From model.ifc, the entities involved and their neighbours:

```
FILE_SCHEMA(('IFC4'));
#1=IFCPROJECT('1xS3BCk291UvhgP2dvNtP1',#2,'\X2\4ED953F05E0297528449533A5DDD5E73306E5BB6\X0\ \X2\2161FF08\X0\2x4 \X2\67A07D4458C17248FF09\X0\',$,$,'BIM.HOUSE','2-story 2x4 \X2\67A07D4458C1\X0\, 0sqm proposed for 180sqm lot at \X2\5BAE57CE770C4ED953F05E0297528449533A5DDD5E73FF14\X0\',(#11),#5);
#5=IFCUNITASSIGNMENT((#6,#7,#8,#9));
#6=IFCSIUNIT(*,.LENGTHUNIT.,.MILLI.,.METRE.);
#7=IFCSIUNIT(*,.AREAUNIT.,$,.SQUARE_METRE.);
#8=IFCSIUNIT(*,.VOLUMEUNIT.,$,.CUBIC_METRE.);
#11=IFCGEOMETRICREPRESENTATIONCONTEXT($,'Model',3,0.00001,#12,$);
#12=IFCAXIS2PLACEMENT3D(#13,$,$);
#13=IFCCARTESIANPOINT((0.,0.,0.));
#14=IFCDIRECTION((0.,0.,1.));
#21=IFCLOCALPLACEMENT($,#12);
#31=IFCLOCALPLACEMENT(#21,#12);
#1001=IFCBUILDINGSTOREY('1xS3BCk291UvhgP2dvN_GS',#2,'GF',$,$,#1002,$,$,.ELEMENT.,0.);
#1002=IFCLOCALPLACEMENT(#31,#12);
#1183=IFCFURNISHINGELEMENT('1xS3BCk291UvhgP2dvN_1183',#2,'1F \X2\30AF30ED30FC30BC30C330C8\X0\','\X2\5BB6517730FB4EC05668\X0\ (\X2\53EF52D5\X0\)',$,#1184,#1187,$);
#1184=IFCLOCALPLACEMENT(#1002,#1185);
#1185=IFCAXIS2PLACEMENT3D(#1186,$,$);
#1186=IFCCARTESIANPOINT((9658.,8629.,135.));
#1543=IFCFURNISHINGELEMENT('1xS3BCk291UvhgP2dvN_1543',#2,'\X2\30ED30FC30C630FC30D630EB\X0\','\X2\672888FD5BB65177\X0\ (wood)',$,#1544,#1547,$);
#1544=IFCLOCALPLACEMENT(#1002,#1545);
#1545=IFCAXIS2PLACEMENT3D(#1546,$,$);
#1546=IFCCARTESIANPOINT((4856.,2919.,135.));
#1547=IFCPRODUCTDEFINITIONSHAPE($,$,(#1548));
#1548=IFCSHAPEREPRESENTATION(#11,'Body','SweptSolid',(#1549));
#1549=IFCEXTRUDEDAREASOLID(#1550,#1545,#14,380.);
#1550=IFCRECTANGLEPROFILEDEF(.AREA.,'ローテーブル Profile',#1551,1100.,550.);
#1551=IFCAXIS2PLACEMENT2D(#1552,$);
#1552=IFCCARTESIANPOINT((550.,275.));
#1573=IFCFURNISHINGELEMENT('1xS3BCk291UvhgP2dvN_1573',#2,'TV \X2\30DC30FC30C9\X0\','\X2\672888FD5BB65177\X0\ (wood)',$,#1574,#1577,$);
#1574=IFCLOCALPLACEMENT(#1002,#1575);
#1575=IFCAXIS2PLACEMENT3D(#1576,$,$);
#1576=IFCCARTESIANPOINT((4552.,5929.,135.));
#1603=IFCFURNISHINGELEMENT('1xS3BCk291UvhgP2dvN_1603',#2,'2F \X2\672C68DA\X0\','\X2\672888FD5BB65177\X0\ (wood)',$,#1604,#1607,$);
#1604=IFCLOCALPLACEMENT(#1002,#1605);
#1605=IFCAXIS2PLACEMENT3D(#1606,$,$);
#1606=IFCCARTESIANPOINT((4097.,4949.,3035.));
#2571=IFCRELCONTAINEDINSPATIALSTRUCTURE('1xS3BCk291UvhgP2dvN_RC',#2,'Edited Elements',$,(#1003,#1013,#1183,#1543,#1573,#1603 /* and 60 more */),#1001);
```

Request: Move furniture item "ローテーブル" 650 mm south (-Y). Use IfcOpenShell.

```python
import ifcopenshell
import ifcopenshell.api.geometry
import ifcopenshell.util.placement

model = ifcopenshell.open("model.ifc")

item = model.by_guid("1xS3BCk291UvhgP2dvN_1543")
matrix = ifcopenshell.util.placement.get_local_placement(item.ObjectPlacement)
matrix[1, 3] -= 650.0
ifcopenshell.api.geometry.edit_object_placement(model, product=item, matrix=matrix, is_si=False)

print(ifcopenshell.util.placement.get_local_placement(item.ObjectPlacement).round(3) + 0.0)

model.write("model_v2.ifc")
```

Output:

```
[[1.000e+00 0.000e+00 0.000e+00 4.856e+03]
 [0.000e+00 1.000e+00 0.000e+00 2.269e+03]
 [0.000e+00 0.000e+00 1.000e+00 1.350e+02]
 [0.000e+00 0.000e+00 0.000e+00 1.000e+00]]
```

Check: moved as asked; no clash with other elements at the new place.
